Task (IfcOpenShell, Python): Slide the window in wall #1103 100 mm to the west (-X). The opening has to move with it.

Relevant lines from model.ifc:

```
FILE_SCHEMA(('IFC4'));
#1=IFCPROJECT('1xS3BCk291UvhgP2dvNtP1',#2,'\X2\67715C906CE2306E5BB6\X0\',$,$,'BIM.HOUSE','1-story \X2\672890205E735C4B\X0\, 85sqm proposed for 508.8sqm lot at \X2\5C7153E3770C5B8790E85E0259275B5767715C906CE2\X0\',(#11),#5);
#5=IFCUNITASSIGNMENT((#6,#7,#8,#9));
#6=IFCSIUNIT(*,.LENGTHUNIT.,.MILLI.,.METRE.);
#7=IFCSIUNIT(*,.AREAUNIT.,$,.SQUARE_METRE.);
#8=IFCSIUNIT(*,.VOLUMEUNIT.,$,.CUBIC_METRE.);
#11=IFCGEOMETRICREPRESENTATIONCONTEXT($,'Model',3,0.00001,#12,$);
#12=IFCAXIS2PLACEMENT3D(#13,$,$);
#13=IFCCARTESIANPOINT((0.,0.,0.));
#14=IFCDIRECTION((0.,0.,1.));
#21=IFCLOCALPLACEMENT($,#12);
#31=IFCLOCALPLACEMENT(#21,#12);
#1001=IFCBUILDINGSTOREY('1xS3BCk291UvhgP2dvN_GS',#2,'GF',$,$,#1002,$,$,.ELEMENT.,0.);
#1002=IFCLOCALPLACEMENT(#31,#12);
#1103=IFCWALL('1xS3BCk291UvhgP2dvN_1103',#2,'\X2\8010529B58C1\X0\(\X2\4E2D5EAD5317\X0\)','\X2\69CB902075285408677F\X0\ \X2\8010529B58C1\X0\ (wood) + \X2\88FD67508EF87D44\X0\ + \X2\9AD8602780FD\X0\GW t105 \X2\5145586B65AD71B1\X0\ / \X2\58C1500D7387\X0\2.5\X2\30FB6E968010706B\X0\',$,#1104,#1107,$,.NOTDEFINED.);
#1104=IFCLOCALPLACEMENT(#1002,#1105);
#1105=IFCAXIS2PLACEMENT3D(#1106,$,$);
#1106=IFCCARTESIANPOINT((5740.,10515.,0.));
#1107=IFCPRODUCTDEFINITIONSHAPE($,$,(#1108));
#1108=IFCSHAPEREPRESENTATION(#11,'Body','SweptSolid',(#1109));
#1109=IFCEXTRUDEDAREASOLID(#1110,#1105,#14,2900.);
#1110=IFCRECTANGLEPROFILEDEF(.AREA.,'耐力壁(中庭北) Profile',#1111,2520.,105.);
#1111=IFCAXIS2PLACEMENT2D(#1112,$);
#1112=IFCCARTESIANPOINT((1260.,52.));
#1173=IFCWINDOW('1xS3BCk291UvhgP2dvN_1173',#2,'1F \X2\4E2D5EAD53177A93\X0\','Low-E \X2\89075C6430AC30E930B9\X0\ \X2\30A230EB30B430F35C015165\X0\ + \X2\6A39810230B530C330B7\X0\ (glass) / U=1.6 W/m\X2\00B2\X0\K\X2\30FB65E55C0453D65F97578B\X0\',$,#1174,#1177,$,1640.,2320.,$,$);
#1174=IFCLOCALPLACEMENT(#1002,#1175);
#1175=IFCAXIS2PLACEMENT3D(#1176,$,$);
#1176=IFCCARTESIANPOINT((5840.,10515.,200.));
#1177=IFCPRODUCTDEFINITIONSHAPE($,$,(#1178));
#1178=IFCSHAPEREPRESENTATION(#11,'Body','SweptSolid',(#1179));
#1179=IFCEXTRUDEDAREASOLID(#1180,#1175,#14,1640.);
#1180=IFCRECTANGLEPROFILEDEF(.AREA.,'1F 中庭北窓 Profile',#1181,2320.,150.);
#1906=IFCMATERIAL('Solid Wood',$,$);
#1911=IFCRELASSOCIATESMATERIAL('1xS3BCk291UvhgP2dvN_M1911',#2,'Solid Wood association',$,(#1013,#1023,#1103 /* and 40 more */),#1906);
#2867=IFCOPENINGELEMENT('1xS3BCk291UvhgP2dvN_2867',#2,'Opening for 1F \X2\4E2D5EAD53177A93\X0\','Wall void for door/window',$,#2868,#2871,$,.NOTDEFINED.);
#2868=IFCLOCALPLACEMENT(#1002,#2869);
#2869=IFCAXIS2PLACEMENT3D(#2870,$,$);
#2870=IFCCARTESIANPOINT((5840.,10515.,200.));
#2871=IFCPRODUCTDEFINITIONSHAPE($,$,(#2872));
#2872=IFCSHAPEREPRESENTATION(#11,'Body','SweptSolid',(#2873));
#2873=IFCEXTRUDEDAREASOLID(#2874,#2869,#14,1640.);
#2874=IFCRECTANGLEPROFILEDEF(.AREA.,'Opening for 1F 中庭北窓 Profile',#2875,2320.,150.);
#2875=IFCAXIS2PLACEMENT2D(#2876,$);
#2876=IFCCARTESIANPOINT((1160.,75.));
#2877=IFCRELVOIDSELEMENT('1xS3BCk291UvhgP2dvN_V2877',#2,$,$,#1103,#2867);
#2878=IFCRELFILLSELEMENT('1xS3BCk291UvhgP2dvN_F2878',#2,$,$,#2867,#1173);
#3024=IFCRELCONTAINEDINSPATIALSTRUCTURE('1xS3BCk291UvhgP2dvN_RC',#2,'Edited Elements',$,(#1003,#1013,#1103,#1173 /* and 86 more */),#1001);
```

```python
import ifcopenshell
import ifcopenshell.api.geometry
import ifcopenshell.util.placement

model = ifcopenshell.open("model.ifc")

window = model.by_guid("1xS3BCk291UvhgP2dvN_1173")
opening = window.FillsVoids[0].RelatingOpeningElement
wall = opening.VoidsElements[0].RelatingBuildingElement

wall_matrix = ifcopenshell.util.placement.get_local_placement(wall.ObjectPlacement)
shift = wall_matrix[:3, 0] * -100.0
before = ifcopenshell.util.placement.get_local_placement(window.ObjectPlacement)[:3, 3].copy()

# The window is not placed relative to its opening, so move both.
for product in (opening, window):
    matrix = ifcopenshell.util.placement.get_local_placement(product.ObjectPlacement)
    matrix[:3, 3] += shift
    ifcopenshell.api.geometry.edit_object_placement(model, product=product, matrix=matrix, is_si=False)

after = ifcopenshell.util.placement.get_local_placement(window.ObjectPlacement)[:3, 3]
print("window moved by", (after - before).round(3) + 0.0)

model.write("model_updated.ifc")
```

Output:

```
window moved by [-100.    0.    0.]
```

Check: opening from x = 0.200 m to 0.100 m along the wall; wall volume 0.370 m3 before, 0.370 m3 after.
